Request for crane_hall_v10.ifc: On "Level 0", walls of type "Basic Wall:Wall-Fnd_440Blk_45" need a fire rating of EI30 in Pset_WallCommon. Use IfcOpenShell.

First a look at what the model holds.

```python
import ifcopenshell
import ifcopenshell.util.element

model = ifcopenshell.open("crane_hall_v10.ifc")
print(model.schema)
storey = next(s for s in model.by_type("IfcBuildingStorey") if s.Name == "Level 0")
walls = [e for e in ifcopenshell.util.element.get_decomposition(storey) if e.is_a("IfcWall")]
seen = {}
for e in walls:
    element_type = ifcopenshell.util.element.get_type(e)
    key = (element_type.Name if element_type != e and element_type else None, ifcopenshell.util.element.get_pset(e, "Pset_WallCommon", "FireRating"))
    seen[key] = seen.get(key, 0) + 1
for (name, value), count in sorted(seen.items(), key=str):
    print(count, "x", name, "|", value)
```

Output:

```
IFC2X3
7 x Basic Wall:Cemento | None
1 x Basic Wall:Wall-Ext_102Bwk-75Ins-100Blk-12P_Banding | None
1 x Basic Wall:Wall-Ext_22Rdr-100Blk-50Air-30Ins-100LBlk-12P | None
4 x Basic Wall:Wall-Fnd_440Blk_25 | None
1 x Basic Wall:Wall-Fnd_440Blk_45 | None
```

```python
import ifcopenshell
import ifcopenshell.api.pset
import ifcopenshell.util.element

model = ifcopenshell.open("crane_hall_v10.ifc")

storey = next(s for s in model.by_type("IfcBuildingStorey") if s.Name == "Level 0")
walls = [e for e in ifcopenshell.util.element.get_decomposition(storey) if e.is_a("IfcWall")]

count = 0
for e in walls:
    element_type = ifcopenshell.util.element.get_type(e)
    if element_type in (None, e) or element_type.Name != "Basic Wall:Wall-Fnd_440Blk_45":
        continue
    # add_pset returns the element's existing set when there is one.
    pset = ifcopenshell.api.pset.add_pset(model, product=e, name="Pset_WallCommon")
    ifcopenshell.api.pset.edit_pset(model, pset=pset, properties={"FireRating": "EI30"})
    count += 1

print(count, "walls updated")

model.write("crane_hall_v10_edited.ifc")
```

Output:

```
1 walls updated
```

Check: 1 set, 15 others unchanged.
